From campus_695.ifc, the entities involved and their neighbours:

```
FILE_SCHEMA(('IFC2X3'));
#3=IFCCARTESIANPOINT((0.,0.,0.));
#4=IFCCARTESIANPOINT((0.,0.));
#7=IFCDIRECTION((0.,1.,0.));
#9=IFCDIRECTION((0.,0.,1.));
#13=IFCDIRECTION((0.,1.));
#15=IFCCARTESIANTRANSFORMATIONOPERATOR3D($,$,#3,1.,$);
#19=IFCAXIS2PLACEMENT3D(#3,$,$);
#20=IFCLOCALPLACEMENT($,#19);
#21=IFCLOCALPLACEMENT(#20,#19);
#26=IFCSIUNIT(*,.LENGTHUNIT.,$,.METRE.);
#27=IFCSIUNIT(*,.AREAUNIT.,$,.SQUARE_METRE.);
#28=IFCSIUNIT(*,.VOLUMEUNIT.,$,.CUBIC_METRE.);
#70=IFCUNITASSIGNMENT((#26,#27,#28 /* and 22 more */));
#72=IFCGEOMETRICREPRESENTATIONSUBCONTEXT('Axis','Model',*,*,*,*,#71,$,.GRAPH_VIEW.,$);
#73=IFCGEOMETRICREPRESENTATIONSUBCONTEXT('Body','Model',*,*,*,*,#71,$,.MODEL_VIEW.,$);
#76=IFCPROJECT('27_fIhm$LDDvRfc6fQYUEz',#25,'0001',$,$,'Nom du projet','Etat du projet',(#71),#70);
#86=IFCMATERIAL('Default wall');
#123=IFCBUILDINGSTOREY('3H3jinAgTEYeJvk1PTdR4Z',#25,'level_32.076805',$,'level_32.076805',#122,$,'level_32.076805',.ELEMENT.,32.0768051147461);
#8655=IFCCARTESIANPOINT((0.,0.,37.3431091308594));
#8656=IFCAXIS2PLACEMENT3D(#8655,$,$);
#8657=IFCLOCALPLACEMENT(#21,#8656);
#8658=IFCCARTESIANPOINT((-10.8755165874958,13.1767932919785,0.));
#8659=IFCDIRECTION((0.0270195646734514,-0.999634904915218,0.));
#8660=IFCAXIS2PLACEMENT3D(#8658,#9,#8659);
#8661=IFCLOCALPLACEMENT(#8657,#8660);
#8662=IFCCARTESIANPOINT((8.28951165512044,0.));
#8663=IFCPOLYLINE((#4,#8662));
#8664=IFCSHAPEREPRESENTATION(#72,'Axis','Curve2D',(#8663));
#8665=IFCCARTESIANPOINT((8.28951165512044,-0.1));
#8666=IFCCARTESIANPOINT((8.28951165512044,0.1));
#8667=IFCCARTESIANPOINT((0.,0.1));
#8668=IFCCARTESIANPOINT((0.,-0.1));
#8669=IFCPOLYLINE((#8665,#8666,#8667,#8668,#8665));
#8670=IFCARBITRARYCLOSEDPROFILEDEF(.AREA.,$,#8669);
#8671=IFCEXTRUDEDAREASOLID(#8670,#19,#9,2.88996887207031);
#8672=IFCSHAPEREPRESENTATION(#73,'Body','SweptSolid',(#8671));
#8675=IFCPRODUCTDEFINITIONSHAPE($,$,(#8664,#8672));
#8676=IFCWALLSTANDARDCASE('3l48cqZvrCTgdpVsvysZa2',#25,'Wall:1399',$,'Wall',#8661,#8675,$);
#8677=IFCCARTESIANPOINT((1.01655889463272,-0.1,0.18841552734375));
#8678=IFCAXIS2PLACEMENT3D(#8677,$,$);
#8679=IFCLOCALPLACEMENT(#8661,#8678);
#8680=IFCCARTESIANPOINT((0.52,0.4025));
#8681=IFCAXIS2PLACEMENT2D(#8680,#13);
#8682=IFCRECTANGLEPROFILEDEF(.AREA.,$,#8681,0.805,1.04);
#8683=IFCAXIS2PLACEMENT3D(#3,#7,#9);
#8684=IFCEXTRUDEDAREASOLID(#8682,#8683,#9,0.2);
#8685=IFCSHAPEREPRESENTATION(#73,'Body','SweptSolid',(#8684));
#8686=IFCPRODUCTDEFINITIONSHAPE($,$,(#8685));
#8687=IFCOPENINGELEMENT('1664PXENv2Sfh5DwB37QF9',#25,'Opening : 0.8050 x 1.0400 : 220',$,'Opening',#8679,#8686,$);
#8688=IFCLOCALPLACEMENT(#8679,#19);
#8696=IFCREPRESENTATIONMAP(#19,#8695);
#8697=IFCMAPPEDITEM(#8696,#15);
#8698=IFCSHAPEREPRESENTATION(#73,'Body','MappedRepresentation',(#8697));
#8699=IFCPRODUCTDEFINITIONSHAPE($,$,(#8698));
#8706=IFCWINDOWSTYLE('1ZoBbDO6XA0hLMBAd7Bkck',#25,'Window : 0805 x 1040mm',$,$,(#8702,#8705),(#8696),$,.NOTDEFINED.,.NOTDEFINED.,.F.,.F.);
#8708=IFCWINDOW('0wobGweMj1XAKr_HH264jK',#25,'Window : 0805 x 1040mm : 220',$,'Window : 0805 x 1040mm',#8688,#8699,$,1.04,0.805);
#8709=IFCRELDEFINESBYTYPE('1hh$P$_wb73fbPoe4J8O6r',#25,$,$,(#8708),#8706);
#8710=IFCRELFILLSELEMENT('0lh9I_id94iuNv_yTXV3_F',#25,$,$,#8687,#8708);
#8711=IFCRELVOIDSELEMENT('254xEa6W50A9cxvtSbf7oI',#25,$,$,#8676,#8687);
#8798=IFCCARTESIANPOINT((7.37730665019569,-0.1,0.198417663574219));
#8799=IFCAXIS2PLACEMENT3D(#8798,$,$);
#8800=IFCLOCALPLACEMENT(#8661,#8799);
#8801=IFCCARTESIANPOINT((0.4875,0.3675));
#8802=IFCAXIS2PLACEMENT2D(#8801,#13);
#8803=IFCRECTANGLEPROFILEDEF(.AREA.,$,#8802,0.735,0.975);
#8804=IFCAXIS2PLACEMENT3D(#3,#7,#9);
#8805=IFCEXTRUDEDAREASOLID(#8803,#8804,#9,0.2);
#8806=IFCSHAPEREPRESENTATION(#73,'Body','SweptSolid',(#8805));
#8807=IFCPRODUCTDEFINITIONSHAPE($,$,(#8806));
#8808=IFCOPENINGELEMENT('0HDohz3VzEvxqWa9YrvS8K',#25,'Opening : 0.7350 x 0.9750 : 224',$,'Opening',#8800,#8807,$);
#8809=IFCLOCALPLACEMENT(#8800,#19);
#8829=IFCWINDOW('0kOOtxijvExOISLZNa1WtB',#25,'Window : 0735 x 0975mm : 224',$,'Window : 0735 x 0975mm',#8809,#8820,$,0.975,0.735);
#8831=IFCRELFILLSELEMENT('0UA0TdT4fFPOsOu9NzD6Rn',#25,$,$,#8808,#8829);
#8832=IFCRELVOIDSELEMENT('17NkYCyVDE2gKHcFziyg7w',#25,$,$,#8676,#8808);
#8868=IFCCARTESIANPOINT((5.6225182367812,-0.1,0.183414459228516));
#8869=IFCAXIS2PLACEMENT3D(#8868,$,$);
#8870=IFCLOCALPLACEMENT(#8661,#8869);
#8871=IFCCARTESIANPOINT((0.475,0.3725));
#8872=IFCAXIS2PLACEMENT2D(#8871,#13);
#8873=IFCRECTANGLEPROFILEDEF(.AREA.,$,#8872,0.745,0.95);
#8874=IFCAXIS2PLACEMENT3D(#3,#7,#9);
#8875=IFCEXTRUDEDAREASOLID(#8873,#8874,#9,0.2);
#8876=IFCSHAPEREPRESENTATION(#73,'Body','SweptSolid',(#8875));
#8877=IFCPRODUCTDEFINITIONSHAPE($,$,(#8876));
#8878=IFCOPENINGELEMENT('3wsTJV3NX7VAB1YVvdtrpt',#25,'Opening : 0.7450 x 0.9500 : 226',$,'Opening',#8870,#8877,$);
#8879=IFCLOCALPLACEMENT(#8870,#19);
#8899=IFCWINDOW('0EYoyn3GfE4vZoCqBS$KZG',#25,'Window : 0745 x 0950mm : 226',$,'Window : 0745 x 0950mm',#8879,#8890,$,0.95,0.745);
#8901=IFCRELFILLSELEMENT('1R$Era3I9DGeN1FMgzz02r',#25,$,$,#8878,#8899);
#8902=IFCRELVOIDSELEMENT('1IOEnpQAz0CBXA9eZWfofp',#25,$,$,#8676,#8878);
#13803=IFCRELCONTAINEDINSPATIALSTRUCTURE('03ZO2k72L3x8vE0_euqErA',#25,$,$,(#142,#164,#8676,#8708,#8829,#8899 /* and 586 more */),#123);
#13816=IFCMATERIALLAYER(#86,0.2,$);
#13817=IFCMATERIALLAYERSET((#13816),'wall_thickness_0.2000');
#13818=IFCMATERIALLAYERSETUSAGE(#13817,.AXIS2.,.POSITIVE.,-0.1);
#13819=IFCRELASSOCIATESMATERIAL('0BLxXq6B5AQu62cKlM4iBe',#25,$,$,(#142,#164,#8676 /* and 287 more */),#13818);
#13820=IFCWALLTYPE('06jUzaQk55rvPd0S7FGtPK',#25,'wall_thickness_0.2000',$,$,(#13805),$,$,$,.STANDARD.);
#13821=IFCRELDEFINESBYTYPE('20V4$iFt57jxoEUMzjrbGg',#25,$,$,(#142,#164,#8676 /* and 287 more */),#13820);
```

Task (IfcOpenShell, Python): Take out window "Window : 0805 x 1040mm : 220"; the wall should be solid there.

```python
import ifcopenshell
import ifcopenshell.api.feature
import ifcopenshell.api.root
import ifcopenshell.geom
import ifcopenshell.util.shape

model = ifcopenshell.open("campus_695.ifc")
settings = ifcopenshell.geom.settings()


def volume(element):
    """Net volume in cubic metres, openings subtracted."""
    shape = ifcopenshell.geom.create_shape(settings, element)
    return ifcopenshell.util.shape.get_volume(shape.geometry)


window = model.by_guid("0wobGweMj1XAKr_HH264jK")
opening = window.FillsVoids[0].RelatingOpeningElement
wall = opening.VoidsElements[0].RelatingBuildingElement
before = volume(wall)

ifcopenshell.api.root.remove_product(model, product=window)
ifcopenshell.api.feature.remove_feature(model, feature=opening)

after = volume(wall)

print(f"wall volume {before:.3f} -> {after:.3f} m3")

model.write("campus_695_edited.ifc")
```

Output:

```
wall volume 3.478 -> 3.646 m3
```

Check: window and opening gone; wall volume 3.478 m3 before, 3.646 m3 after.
